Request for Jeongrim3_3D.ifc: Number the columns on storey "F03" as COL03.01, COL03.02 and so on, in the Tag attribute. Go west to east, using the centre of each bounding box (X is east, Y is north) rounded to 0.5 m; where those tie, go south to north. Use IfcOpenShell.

First a look at what the model holds.

```python
import ifcopenshell
import ifcopenshell.util.element
import ifcopenshell.util.placement

model = ifcopenshell.open("Jeongrim3_3D.ifc")
print(model.schema)
storey = next(s for s in model.by_type("IfcBuildingStorey") if s.Name == "F03")
columns = [e for e in ifcopenshell.util.element.get_decomposition(storey) if e.is_a("IfcColumn")]
for e in sorted(columns, key=lambda e: e.id()):
    origin = ifcopenshell.util.placement.get_local_placement(e.ObjectPlacement)[:3, 3]
    print(e.id(), e.Tag, e.Name, origin.round(2) + 0.0, sep=" | ")
```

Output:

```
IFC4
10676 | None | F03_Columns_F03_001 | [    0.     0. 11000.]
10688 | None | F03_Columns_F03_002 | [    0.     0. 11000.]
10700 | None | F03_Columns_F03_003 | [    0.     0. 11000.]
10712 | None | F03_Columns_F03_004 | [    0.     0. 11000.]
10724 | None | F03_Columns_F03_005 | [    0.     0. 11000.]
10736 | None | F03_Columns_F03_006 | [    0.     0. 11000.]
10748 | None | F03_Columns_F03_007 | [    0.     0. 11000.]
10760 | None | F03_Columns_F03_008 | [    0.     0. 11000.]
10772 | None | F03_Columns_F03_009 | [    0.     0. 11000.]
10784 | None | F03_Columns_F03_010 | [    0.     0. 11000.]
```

```python
import ifcopenshell
import ifcopenshell.geom
import ifcopenshell.util.element
import ifcopenshell.util.shape

model = ifcopenshell.open("Jeongrim3_3D.ifc")
settings = ifcopenshell.geom.settings()
settings.set("use-world-coords", True)


def centre(element):
    shape = ifcopenshell.geom.create_shape(settings, element)
    return ifcopenshell.util.shape.get_bbox_centroid(shape.geometry)


storey = next(s for s in model.by_type("IfcBuildingStorey") if s.Name == "F03")
columns = [e for e in ifcopenshell.util.element.get_decomposition(storey) if e.is_a("IfcColumn")]

# Insertion points can sit at a corner or the storey origin, so sort by the geometry (in metres).
centres = {e: centre(e) for e in columns}
columns.sort(key=lambda e: (round(centres[e][0] / 0.5), centres[e][1]))

for i, e in enumerate(columns, start=1):
    number = f"COL03.{i:02d}"
    e.Tag = number
    print(e.id(), number)

model.write("Jeongrim3_3D_v2.ifc")
```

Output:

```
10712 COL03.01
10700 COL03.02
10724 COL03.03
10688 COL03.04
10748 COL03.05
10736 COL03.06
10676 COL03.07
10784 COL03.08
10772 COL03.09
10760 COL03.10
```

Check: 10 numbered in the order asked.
